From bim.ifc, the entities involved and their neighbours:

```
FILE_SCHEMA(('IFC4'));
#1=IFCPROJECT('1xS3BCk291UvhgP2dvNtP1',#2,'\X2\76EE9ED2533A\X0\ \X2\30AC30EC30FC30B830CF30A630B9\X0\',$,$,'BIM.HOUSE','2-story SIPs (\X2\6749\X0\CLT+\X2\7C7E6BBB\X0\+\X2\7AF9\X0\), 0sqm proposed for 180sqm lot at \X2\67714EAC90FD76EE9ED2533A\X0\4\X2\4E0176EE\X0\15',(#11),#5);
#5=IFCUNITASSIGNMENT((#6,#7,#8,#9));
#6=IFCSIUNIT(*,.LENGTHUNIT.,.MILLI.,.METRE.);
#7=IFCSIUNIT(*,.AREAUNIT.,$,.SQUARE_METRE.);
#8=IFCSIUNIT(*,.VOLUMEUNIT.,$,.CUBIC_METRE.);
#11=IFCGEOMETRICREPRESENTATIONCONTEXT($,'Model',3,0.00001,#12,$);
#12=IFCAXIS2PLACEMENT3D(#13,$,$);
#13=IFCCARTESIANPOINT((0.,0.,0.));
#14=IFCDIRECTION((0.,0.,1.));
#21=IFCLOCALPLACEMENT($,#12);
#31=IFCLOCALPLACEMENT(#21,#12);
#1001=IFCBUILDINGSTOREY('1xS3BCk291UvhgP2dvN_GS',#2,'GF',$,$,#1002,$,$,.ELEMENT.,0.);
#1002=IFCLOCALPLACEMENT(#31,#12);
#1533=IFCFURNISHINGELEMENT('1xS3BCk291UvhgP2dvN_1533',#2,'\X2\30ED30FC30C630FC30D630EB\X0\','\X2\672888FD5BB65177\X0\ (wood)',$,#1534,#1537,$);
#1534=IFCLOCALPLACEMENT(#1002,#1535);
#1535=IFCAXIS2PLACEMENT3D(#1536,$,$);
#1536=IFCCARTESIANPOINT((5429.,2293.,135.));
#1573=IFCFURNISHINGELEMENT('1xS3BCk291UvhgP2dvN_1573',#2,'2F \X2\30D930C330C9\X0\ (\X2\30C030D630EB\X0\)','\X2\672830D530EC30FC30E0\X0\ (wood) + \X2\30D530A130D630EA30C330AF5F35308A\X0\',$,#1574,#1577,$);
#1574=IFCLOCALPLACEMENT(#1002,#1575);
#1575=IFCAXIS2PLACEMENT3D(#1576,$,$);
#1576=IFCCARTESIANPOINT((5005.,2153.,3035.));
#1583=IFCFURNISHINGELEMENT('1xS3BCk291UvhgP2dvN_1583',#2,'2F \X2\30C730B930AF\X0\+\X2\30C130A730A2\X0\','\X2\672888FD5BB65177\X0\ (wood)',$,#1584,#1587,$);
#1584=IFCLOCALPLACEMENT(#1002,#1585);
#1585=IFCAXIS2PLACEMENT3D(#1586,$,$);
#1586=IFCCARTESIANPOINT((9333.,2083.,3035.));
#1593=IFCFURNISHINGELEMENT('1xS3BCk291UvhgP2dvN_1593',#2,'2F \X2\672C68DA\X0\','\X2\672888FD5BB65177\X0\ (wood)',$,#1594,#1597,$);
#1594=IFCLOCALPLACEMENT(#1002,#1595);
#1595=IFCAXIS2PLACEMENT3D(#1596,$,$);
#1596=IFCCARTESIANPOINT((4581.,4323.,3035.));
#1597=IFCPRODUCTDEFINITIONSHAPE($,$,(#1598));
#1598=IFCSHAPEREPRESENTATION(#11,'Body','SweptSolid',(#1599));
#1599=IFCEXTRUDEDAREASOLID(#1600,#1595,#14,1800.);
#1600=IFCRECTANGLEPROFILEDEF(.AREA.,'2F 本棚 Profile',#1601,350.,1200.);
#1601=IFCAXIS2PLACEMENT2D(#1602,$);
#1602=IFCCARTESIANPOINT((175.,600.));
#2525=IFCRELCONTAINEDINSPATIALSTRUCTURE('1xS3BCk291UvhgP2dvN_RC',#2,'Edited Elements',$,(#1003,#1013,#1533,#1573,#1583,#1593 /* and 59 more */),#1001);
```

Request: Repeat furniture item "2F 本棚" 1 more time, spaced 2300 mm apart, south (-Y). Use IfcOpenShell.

```python
import numpy as np
import ifcopenshell
import ifcopenshell.api.geometry
import ifcopenshell.api.root
import ifcopenshell.util.element
import ifcopenshell.util.placement

model = ifcopenshell.open("bim.ifc")


def reuse_history(source, copy):
    """copy_class also copies each property set's owner history, people and application; keep the originals."""
    for rel in copy.IsDefinedBy:
        if rel.is_a("IfcRelDefinesByProperties") and (history := rel.RelatingPropertyDefinition.OwnerHistory):
            rel.RelatingPropertyDefinition.OwnerHistory = source.OwnerHistory
            ifcopenshell.util.element.remove_deep2(model, history)


source = model.by_guid("1xS3BCk291UvhgP2dvN_1593")
base = ifcopenshell.util.placement.get_local_placement(source.ObjectPlacement)
step = np.array([0.0, -1.0, 0.0]) * 2300.0

for i in range(1, 2):
    copy = ifcopenshell.api.root.copy_class(model, product=source)
    copy.Representation = ifcopenshell.util.element.copy_deep(
        model, source.Representation, exclude=["IfcGeometricRepresentationContext", "IfcRepresentationMap"]
    )
    reuse_history(source, copy)
    matrix = base.copy()
    matrix[:3, 3] += i * step
    print("added at", matrix[:3, 3].round(3) + 0.0)
    ifcopenshell.api.geometry.edit_object_placement(model, product=copy, matrix=matrix, is_si=False)

model.write("bim_updated.ifc")
```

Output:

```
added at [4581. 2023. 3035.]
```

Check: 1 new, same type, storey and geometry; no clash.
